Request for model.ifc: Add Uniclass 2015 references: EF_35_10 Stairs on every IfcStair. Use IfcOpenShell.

First a look at what the model holds.

```python
import ifcopenshell

model = ifcopenshell.open("model.ifc")
print(model.schema)
print("classifications:", [c.Name for c in model.by_type("IfcClassification")])
for ifc_class in ("IfcDoor", "IfcRoof", "IfcStair", "IfcWall", "IfcWindow"):
    print(ifc_class, len(model.by_type(ifc_class)))
```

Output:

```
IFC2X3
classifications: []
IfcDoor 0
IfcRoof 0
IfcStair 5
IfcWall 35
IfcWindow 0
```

```python
import ifcopenshell
import ifcopenshell.api.classification

model = ifcopenshell.open("model.ifc")

# IFC2X3 requires Source and Edition and has no link from the project to the system.
system = model.create_entity("IfcClassification", Source="NBS", Edition="2015", Name="Uniclass 2015")

codes = {
    "IfcStair": ("EF_35_10", "Stairs"),
}
for ifc_class, (code, name) in codes.items():
    products = model.by_type(ifc_class)
    ifcopenshell.api.classification.add_reference(
        model, products=products, classification=system, identification=code, name=name
    )
    print(code, len(products))

model.write("model_rev.ifc")
```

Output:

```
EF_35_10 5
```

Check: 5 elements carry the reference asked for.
